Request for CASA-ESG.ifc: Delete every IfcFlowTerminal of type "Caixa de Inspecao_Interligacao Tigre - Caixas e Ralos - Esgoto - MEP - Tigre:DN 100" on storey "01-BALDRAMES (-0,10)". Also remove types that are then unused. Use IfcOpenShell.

First a look at what the model holds.

```python
import ifcopenshell
import ifcopenshell.util.element

model = ifcopenshell.open("CASA-ESG.ifc")
print(model.schema)
storey = next(s for s in model.by_type("IfcBuildingStorey") if s.Name == "01-BALDRAMES (-0,10)")
terminals = [e for e in ifcopenshell.util.element.get_decomposition(storey) if e.is_a("IfcFlowTerminal")]
seen = {}
for e in terminals:
    element_type = ifcopenshell.util.element.get_type(e)
    name = element_type.Name if element_type not in (None, e) else None
    seen[name] = seen.get(name, 0) + 1
for name, count in sorted(seen.items(), key=str):
    print(count, "x", name)
```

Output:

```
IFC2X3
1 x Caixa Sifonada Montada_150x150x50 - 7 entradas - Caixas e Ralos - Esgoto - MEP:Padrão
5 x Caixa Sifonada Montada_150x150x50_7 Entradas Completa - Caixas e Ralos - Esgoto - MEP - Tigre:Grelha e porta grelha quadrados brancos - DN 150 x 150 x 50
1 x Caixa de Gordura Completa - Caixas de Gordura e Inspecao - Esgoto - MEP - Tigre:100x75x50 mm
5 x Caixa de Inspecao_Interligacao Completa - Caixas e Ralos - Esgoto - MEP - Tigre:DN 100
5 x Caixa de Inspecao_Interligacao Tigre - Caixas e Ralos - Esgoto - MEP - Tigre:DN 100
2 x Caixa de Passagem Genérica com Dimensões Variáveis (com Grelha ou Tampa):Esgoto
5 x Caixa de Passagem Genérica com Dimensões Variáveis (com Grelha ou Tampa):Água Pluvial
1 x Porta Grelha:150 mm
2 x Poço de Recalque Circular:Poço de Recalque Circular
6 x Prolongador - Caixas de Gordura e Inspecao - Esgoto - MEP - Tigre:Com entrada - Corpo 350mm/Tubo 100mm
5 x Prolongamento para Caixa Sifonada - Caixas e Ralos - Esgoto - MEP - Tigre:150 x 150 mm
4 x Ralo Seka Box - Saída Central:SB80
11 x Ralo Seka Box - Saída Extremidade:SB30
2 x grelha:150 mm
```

```python
import ifcopenshell
import ifcopenshell.api.root
import ifcopenshell.util.element

model = ifcopenshell.open("CASA-ESG.ifc")

storey = next(s for s in model.by_type("IfcBuildingStorey") if s.Name == "01-BALDRAMES (-0,10)")
terminals = [e for e in ifcopenshell.util.element.get_decomposition(storey) if e.is_a("IfcFlowTerminal")]
targets = [e for e in terminals if (t := ifcopenshell.util.element.get_type(e)) not in (None, e) and t.Name == "Caixa de Inspecao_Interligacao Tigre - Caixas e Ralos - Esgoto - MEP - Tigre:DN 100"]
types = {ifcopenshell.util.element.get_type(e) for e in targets} - {None, *targets}

for e in targets:
    ifcopenshell.api.root.remove_product(model, product=e)
print(len(targets), "removed")

unused = [t for t in types if not ifcopenshell.util.element.get_types(t)]
for t in unused:
    ifcopenshell.api.root.remove_product(model, product=t)
print(len(unused), "unused types removed")

model.write("CASA-ESG_updated.ifc")
```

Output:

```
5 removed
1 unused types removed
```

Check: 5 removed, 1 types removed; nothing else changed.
